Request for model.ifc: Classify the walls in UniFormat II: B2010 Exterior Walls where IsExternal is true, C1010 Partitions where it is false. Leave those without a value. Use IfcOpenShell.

First a look at what the model holds.

```python
import ifcopenshell
import ifcopenshell.util.element

model = ifcopenshell.open("model.ifc")
print(model.schema)
print("classifications:", [c.Name for c in model.by_type("IfcClassification")])
values = [ifcopenshell.util.element.get_pset(e, "Pset_WallCommon", "IsExternal") for e in model.by_type("IfcWall")]
for value in (True, False, None):
    print("IsExternal", value, values.count(value))
```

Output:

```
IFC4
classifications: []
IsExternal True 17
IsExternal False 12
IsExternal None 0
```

```python
import ifcopenshell
import ifcopenshell.api.classification
import ifcopenshell.util.element

model = ifcopenshell.open("model.ifc")

system = ifcopenshell.api.classification.add_classification(model, classification="UniFormat II")

walls = model.by_type("IfcWall")
external = {e: ifcopenshell.util.element.get_pset(e, "Pset_WallCommon", "IsExternal") for e in walls}
for flag, code, name in ((True, "B2010", "Exterior Walls"), (False, "C1010", "Partitions")):
    products = [e for e in walls if external[e] is flag]
    ifcopenshell.api.classification.add_reference(
        model, products=products, classification=system, identification=code, name=name
    )
    print(code, len(products))

model.write("model_v2.ifc")
```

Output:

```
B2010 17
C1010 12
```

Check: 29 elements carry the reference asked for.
